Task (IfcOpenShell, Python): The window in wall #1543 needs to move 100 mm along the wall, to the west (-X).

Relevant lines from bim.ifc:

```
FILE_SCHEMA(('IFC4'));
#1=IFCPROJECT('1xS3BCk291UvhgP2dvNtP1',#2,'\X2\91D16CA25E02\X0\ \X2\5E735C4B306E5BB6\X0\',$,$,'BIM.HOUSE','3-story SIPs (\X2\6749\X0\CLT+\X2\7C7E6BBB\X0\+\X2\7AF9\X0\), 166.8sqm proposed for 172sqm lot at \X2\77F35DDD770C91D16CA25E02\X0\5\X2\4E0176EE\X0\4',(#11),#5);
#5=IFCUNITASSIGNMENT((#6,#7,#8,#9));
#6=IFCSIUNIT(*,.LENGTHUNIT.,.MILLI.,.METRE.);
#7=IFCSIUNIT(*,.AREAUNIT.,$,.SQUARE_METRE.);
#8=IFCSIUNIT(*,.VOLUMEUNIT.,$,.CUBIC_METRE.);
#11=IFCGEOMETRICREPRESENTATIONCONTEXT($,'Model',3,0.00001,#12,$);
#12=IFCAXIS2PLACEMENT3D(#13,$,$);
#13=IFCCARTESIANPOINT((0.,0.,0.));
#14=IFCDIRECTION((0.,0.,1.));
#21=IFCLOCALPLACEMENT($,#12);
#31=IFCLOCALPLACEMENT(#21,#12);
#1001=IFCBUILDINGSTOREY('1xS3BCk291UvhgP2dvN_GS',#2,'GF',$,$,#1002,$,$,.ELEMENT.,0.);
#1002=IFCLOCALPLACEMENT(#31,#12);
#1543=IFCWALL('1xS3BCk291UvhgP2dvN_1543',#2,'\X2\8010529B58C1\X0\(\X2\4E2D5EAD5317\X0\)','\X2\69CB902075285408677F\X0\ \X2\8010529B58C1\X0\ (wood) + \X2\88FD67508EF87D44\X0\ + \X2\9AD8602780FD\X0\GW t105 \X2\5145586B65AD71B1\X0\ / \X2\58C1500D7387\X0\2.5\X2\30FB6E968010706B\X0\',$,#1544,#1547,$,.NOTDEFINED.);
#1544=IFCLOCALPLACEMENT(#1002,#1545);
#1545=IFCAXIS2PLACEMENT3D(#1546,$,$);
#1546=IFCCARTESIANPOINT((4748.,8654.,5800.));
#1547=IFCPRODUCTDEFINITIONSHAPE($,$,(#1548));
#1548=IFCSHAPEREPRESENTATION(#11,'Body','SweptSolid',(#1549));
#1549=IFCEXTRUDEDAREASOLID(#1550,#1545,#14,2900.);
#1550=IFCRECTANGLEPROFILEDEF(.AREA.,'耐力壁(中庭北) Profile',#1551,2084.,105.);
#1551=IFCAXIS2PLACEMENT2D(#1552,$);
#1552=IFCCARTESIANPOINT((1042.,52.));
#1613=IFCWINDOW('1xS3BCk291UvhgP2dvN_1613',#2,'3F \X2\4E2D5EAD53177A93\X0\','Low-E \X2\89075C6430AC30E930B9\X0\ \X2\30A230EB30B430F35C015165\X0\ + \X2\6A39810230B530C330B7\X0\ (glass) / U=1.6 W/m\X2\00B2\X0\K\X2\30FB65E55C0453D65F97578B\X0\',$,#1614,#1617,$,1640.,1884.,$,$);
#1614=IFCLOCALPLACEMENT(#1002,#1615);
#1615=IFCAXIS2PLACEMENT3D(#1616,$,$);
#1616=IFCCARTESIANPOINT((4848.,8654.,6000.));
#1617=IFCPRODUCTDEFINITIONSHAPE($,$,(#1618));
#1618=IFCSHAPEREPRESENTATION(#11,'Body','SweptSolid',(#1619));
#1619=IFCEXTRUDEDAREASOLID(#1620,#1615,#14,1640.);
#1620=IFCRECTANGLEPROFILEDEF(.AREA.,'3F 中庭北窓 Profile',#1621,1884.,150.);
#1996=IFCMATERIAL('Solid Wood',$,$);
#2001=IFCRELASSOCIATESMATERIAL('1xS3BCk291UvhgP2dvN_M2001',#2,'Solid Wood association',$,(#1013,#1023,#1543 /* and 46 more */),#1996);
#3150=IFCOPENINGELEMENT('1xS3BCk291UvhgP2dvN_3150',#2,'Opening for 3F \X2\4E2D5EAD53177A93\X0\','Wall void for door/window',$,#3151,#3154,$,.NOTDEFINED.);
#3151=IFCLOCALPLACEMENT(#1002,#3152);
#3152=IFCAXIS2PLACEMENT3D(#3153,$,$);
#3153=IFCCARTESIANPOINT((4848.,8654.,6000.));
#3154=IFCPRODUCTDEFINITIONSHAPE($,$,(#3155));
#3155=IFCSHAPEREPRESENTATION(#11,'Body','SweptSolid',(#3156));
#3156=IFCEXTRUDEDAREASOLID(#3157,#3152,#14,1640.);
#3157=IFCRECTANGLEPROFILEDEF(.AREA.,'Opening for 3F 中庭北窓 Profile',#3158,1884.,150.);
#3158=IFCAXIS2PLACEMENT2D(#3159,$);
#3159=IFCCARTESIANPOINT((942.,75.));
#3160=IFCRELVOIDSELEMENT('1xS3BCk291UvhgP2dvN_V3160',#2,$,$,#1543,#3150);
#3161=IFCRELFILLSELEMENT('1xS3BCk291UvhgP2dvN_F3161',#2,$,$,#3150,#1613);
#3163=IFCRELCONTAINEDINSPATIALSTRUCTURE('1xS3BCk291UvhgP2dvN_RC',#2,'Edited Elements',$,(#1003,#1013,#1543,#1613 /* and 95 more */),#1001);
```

```python
import ifcopenshell
import ifcopenshell.api.geometry
import ifcopenshell.util.placement
import ifcopenshell.util.unit

model = ifcopenshell.open("bim.ifc")
unit_scale = ifcopenshell.util.unit.calculate_unit_scale(model)

window = model.by_guid("1xS3BCk291UvhgP2dvN_1613")
opening = window.FillsVoids[0].RelatingOpeningElement
wall = opening.VoidsElements[0].RelatingBuildingElement

wall_matrix = ifcopenshell.util.placement.get_local_placement(wall.ObjectPlacement)
shift = wall_matrix[:3, 0] * -0.1 / unit_scale
before = ifcopenshell.util.placement.get_local_placement(window.ObjectPlacement)[:3, 3].copy()

# The window is not placed relative to its opening, so move both.
for product in (opening, window):
    matrix = ifcopenshell.util.placement.get_local_placement(product.ObjectPlacement)
    matrix[:3, 3] += shift
    ifcopenshell.api.geometry.edit_object_placement(model, product=product, matrix=matrix, is_si=False)

after = ifcopenshell.util.placement.get_local_placement(window.ObjectPlacement)[:3, 3]
print("window moved by", (after - before).round(3) + 0.0)

model.write("bim_updated.ifc")
```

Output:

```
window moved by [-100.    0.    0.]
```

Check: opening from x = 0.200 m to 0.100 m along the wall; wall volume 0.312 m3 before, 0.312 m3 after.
